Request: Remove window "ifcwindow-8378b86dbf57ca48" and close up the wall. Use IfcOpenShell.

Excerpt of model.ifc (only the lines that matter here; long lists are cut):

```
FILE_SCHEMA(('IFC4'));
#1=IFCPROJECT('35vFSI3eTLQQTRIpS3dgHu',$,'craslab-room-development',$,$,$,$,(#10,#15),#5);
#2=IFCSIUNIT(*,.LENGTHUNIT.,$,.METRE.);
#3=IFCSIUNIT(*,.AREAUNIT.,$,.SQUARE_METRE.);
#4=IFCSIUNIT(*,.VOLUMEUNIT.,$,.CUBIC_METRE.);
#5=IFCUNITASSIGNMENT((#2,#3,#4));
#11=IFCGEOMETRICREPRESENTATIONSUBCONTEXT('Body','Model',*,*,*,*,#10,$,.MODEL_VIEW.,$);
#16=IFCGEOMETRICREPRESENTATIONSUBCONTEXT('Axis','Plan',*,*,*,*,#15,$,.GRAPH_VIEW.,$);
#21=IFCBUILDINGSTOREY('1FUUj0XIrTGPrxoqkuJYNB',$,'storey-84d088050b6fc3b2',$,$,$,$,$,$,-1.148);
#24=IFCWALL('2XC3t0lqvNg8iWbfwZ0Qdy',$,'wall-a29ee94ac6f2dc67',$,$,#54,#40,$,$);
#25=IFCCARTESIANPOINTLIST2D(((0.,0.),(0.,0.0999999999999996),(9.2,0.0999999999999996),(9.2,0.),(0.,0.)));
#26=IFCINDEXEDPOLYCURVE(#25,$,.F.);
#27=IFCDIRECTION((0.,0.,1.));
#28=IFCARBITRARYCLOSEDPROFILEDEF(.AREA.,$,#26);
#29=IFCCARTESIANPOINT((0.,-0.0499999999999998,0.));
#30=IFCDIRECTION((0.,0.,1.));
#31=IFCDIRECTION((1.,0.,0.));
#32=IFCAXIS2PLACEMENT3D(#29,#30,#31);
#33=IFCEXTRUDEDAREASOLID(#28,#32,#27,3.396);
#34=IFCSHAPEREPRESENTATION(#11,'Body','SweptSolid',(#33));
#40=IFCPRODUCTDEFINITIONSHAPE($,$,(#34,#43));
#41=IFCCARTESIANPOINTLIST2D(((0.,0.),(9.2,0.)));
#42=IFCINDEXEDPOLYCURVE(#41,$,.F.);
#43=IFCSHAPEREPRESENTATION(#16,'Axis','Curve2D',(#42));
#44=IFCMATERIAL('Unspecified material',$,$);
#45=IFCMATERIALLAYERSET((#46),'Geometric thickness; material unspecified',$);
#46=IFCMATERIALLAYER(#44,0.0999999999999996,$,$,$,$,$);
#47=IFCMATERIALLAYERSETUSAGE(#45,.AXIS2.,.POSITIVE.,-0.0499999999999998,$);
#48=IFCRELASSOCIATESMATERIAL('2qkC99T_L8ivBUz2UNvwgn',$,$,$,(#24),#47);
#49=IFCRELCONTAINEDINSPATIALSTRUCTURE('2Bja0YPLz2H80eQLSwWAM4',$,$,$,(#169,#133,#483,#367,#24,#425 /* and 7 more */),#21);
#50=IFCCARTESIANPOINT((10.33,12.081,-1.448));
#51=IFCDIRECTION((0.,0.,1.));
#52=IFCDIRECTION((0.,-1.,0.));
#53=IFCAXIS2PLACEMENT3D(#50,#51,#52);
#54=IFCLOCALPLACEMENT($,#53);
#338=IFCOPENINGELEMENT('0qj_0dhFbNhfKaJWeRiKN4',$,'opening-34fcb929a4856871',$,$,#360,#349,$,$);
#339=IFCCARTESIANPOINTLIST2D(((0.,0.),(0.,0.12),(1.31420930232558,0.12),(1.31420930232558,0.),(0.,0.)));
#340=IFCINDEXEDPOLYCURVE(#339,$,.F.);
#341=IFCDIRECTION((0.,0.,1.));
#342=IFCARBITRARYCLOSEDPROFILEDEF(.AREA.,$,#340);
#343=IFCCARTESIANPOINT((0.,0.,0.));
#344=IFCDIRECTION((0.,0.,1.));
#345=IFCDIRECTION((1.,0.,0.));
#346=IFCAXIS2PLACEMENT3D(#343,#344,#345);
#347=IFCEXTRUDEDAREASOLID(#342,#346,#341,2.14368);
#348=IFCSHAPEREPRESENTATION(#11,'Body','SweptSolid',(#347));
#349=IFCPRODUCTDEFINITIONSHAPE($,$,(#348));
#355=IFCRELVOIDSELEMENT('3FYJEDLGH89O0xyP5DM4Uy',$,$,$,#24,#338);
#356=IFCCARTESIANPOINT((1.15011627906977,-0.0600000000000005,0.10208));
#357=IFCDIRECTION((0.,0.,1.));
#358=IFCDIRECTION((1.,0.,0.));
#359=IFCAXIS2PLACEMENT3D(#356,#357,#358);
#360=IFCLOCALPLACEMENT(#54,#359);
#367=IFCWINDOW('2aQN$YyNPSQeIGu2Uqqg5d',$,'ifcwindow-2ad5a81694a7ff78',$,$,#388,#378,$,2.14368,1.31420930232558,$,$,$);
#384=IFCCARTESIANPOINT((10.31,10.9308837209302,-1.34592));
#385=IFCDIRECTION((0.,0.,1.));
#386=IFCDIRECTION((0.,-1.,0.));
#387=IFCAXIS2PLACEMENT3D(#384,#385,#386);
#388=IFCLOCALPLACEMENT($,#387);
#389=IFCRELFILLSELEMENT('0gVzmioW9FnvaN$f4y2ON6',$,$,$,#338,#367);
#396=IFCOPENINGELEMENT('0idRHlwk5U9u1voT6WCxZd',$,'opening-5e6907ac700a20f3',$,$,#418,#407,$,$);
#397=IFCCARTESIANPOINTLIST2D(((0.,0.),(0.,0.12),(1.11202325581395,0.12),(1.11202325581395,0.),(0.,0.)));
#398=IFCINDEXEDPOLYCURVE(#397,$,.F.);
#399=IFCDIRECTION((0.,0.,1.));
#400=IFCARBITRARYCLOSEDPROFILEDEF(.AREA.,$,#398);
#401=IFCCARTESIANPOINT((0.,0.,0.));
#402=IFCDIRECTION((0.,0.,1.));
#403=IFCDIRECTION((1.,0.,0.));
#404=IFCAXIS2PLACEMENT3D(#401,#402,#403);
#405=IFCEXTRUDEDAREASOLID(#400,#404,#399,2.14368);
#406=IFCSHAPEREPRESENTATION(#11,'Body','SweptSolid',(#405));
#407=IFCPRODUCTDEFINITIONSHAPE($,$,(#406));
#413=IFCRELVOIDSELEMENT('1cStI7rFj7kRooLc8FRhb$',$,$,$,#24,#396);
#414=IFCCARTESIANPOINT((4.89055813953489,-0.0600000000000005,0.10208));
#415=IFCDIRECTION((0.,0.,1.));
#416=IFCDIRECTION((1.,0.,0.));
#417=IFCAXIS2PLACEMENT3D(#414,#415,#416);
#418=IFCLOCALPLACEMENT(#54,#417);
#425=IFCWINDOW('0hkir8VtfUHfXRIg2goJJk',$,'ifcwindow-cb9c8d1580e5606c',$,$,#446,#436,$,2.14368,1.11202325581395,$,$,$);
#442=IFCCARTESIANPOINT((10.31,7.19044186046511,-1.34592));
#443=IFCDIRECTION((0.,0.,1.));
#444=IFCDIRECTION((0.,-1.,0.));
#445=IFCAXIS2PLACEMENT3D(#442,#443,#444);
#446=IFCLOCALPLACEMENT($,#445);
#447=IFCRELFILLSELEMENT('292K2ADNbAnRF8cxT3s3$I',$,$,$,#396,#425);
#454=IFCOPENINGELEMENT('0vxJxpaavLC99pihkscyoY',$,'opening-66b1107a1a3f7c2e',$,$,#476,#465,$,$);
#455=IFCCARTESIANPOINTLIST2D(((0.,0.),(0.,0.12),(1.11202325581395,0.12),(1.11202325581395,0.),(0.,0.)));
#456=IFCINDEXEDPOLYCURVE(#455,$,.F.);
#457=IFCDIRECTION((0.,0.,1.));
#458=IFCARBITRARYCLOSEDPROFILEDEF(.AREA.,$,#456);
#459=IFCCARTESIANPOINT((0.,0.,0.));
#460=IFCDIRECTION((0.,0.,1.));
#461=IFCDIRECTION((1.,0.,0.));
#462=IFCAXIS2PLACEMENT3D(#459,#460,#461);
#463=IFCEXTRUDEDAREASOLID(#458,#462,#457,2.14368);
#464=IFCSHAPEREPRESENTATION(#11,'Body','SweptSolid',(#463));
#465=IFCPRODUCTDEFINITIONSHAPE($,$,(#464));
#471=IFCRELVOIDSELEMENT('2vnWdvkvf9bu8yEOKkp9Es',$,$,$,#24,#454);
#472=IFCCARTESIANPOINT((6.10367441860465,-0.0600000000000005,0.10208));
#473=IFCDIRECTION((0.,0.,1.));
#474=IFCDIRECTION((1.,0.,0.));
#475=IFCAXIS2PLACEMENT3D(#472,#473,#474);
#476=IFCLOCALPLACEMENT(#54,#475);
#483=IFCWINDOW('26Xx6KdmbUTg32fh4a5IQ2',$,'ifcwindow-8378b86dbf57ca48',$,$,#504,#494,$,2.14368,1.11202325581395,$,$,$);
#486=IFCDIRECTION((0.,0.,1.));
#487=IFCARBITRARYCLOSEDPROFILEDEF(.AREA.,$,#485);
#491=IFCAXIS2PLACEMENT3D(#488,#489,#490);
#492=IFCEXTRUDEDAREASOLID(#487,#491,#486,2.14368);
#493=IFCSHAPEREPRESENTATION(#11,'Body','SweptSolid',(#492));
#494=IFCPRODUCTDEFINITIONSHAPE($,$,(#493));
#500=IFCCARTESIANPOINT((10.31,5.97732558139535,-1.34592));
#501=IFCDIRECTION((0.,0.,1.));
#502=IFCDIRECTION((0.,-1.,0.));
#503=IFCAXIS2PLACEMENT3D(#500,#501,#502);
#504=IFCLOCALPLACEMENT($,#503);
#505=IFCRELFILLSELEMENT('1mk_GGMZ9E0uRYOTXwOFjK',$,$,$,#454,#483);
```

```python
import ifcopenshell
import ifcopenshell.api.feature
import ifcopenshell.api.root
import ifcopenshell.geom
import ifcopenshell.util.shape

model = ifcopenshell.open("model.ifc")
settings = ifcopenshell.geom.settings()


def volume(element):
    """Net volume in cubic metres, openings subtracted."""
    shape = ifcopenshell.geom.create_shape(settings, element)
    return ifcopenshell.util.shape.get_volume(shape.geometry)


window = model.by_guid("26Xx6KdmbUTg32fh4a5IQ2")
opening = window.FillsVoids[0].RelatingOpeningElement
wall = opening.VoidsElements[0].RelatingBuildingElement
before = volume(wall)

ifcopenshell.api.root.remove_product(model, product=window)
ifcopenshell.api.feature.remove_feature(model, feature=opening)

after = volume(wall)

print(f"wall volume {before:.3f} -> {after:.3f} m3")

model.write("model_edited.ifc")
```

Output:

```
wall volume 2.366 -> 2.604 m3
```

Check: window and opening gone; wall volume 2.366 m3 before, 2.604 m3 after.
